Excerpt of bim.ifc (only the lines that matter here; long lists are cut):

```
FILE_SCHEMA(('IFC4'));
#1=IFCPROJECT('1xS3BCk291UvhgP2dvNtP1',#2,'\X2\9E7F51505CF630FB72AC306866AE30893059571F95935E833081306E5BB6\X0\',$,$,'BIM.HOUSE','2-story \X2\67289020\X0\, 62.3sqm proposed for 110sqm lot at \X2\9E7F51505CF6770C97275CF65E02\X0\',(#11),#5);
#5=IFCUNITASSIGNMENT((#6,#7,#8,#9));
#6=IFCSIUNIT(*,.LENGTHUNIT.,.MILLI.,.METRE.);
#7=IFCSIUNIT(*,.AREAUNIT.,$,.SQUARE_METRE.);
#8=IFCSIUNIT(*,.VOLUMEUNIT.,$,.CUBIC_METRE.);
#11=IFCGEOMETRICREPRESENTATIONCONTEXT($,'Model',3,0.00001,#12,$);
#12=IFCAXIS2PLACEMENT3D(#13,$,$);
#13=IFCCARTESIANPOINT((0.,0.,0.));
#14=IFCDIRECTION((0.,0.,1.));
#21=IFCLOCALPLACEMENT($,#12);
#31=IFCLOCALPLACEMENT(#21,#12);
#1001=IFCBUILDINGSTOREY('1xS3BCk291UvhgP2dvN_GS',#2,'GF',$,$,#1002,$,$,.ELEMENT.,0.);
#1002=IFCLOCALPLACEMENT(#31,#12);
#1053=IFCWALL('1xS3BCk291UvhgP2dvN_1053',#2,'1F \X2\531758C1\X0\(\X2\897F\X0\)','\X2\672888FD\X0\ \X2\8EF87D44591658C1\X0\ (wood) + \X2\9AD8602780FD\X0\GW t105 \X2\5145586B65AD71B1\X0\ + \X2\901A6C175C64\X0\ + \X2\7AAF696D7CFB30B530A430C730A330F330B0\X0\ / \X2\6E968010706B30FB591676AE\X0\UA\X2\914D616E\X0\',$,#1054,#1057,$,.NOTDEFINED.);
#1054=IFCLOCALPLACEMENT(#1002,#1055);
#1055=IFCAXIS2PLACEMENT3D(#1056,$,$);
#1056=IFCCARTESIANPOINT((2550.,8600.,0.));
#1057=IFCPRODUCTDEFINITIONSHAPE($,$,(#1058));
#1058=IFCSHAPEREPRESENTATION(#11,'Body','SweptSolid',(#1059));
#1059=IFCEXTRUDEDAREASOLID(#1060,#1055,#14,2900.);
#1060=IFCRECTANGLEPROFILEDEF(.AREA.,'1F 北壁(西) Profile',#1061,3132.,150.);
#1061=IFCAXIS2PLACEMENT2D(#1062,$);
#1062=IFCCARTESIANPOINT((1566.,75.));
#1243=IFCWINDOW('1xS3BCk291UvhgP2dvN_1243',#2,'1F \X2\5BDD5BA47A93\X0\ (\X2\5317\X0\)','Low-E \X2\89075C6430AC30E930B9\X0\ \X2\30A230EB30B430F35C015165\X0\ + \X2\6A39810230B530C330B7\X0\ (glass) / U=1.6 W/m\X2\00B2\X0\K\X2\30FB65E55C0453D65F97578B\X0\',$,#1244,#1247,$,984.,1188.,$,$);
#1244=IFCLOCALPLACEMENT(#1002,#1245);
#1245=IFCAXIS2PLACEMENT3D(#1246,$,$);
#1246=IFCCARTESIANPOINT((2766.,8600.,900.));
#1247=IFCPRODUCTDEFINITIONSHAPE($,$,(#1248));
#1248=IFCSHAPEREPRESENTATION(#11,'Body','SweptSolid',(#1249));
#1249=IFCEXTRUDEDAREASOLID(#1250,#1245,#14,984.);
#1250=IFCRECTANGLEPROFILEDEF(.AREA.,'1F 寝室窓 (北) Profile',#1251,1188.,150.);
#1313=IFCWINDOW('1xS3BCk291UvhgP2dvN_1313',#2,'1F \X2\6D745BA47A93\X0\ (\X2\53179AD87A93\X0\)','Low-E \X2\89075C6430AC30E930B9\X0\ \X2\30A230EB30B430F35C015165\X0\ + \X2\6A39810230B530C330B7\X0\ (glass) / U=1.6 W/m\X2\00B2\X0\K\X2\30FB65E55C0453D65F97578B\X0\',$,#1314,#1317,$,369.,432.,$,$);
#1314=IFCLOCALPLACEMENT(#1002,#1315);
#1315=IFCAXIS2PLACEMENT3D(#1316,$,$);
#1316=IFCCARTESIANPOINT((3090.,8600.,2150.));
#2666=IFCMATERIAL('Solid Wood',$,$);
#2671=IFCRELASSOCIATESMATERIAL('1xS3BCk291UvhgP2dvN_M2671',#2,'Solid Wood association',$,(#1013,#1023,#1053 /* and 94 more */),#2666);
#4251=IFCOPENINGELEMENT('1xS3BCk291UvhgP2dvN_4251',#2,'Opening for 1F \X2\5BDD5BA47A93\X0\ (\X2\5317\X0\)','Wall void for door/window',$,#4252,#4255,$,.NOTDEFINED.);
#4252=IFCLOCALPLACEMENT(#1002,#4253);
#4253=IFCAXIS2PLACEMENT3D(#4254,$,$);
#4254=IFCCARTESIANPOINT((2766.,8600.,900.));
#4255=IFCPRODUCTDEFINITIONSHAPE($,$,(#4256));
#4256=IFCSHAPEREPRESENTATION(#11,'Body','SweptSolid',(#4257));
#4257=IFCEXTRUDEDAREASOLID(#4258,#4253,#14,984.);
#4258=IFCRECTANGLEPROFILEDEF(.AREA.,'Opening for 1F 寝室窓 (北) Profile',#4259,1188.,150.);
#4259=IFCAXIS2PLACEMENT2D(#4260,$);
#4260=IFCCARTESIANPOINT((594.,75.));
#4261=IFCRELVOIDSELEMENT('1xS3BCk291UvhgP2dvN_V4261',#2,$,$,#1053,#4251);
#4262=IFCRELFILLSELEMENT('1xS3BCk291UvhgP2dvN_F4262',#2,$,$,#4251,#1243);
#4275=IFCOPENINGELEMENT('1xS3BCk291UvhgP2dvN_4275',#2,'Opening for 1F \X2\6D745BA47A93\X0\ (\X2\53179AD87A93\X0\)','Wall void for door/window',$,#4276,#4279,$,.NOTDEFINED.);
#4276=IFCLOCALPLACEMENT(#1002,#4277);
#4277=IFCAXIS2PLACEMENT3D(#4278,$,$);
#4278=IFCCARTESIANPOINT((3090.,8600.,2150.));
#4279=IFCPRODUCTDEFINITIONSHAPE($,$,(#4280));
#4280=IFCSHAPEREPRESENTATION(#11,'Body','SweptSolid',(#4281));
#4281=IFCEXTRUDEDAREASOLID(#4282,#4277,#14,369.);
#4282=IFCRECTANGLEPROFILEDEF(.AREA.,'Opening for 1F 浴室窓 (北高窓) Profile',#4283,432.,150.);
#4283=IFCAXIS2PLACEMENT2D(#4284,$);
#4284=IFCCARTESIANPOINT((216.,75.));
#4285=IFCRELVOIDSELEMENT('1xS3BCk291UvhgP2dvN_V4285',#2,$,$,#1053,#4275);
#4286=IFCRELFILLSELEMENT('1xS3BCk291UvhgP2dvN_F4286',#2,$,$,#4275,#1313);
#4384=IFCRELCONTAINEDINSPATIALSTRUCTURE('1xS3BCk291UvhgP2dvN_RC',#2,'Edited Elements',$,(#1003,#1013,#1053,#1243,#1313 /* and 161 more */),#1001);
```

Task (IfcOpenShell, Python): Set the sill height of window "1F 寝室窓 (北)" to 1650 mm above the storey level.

```python
import numpy as np
import ifcopenshell
import ifcopenshell.api.geometry
import ifcopenshell.geom
import ifcopenshell.util.element
import ifcopenshell.util.placement
import ifcopenshell.util.shape
import ifcopenshell.util.unit

model = ifcopenshell.open("bim.ifc")
unit_scale = ifcopenshell.util.unit.calculate_unit_scale(model)

window = model.by_guid("1xS3BCk291UvhgP2dvN_1243")
opening = window.FillsVoids[0].RelatingOpeningElement
storey = ifcopenshell.util.element.get_container(window, ifc_class="IfcBuildingStorey")
level = ifcopenshell.util.placement.get_local_placement(storey.ObjectPlacement)[2, 3]

# The opening's origin need not be at the sill, so measure its lowest point.
shape = ifcopenshell.geom.create_shape(ifcopenshell.geom.settings(), opening)
bottom = ifcopenshell.util.shape.get_shape_bottom_elevation(shape, shape.geometry) / unit_scale
dz = level + 1.65 / unit_scale - bottom

shift = np.array([0.0, 0.0, dz])
# The window is not placed relative to its opening, so move both.
for product in (opening, window):
    matrix = ifcopenshell.util.placement.get_local_placement(product.ObjectPlacement)
    matrix[:3, 3] += shift
    ifcopenshell.api.geometry.edit_object_placement(model, product=product, matrix=matrix, is_si=False)

print(f"moved by {dz * unit_scale:+.3f} m")

model.write("bim_updated.ifc")
```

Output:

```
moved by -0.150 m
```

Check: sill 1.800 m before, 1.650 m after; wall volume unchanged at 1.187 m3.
